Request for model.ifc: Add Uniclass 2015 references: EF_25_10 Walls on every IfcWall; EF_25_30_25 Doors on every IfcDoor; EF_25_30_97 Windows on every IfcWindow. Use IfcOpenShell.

First a look at what the model holds.

```python
import ifcopenshell

model = ifcopenshell.open("model.ifc")
print(model.schema)
print("classifications:", [c.Name for c in model.by_type("IfcClassification")])
for ifc_class in ("IfcDoor", "IfcRoof", "IfcStair", "IfcWall", "IfcWindow"):
    print(ifc_class, len(model.by_type(ifc_class)))
```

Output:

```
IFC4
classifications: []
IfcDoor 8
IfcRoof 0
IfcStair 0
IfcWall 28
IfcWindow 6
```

```python
import ifcopenshell
import ifcopenshell.api.classification

model = ifcopenshell.open("model.ifc")

system = ifcopenshell.api.classification.add_classification(model, classification="Uniclass 2015")

codes = {
    "IfcWall": ("EF_25_10", "Walls"),
    "IfcDoor": ("EF_25_30_25", "Doors"),
    "IfcWindow": ("EF_25_30_97", "Windows"),
}
for ifc_class, (code, name) in codes.items():
    products = model.by_type(ifc_class)
    ifcopenshell.api.classification.add_reference(
        model, products=products, classification=system, identification=code, name=name
    )
    print(code, len(products))

model.write("model_rev.ifc")
```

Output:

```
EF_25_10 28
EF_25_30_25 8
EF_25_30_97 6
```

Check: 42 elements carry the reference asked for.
